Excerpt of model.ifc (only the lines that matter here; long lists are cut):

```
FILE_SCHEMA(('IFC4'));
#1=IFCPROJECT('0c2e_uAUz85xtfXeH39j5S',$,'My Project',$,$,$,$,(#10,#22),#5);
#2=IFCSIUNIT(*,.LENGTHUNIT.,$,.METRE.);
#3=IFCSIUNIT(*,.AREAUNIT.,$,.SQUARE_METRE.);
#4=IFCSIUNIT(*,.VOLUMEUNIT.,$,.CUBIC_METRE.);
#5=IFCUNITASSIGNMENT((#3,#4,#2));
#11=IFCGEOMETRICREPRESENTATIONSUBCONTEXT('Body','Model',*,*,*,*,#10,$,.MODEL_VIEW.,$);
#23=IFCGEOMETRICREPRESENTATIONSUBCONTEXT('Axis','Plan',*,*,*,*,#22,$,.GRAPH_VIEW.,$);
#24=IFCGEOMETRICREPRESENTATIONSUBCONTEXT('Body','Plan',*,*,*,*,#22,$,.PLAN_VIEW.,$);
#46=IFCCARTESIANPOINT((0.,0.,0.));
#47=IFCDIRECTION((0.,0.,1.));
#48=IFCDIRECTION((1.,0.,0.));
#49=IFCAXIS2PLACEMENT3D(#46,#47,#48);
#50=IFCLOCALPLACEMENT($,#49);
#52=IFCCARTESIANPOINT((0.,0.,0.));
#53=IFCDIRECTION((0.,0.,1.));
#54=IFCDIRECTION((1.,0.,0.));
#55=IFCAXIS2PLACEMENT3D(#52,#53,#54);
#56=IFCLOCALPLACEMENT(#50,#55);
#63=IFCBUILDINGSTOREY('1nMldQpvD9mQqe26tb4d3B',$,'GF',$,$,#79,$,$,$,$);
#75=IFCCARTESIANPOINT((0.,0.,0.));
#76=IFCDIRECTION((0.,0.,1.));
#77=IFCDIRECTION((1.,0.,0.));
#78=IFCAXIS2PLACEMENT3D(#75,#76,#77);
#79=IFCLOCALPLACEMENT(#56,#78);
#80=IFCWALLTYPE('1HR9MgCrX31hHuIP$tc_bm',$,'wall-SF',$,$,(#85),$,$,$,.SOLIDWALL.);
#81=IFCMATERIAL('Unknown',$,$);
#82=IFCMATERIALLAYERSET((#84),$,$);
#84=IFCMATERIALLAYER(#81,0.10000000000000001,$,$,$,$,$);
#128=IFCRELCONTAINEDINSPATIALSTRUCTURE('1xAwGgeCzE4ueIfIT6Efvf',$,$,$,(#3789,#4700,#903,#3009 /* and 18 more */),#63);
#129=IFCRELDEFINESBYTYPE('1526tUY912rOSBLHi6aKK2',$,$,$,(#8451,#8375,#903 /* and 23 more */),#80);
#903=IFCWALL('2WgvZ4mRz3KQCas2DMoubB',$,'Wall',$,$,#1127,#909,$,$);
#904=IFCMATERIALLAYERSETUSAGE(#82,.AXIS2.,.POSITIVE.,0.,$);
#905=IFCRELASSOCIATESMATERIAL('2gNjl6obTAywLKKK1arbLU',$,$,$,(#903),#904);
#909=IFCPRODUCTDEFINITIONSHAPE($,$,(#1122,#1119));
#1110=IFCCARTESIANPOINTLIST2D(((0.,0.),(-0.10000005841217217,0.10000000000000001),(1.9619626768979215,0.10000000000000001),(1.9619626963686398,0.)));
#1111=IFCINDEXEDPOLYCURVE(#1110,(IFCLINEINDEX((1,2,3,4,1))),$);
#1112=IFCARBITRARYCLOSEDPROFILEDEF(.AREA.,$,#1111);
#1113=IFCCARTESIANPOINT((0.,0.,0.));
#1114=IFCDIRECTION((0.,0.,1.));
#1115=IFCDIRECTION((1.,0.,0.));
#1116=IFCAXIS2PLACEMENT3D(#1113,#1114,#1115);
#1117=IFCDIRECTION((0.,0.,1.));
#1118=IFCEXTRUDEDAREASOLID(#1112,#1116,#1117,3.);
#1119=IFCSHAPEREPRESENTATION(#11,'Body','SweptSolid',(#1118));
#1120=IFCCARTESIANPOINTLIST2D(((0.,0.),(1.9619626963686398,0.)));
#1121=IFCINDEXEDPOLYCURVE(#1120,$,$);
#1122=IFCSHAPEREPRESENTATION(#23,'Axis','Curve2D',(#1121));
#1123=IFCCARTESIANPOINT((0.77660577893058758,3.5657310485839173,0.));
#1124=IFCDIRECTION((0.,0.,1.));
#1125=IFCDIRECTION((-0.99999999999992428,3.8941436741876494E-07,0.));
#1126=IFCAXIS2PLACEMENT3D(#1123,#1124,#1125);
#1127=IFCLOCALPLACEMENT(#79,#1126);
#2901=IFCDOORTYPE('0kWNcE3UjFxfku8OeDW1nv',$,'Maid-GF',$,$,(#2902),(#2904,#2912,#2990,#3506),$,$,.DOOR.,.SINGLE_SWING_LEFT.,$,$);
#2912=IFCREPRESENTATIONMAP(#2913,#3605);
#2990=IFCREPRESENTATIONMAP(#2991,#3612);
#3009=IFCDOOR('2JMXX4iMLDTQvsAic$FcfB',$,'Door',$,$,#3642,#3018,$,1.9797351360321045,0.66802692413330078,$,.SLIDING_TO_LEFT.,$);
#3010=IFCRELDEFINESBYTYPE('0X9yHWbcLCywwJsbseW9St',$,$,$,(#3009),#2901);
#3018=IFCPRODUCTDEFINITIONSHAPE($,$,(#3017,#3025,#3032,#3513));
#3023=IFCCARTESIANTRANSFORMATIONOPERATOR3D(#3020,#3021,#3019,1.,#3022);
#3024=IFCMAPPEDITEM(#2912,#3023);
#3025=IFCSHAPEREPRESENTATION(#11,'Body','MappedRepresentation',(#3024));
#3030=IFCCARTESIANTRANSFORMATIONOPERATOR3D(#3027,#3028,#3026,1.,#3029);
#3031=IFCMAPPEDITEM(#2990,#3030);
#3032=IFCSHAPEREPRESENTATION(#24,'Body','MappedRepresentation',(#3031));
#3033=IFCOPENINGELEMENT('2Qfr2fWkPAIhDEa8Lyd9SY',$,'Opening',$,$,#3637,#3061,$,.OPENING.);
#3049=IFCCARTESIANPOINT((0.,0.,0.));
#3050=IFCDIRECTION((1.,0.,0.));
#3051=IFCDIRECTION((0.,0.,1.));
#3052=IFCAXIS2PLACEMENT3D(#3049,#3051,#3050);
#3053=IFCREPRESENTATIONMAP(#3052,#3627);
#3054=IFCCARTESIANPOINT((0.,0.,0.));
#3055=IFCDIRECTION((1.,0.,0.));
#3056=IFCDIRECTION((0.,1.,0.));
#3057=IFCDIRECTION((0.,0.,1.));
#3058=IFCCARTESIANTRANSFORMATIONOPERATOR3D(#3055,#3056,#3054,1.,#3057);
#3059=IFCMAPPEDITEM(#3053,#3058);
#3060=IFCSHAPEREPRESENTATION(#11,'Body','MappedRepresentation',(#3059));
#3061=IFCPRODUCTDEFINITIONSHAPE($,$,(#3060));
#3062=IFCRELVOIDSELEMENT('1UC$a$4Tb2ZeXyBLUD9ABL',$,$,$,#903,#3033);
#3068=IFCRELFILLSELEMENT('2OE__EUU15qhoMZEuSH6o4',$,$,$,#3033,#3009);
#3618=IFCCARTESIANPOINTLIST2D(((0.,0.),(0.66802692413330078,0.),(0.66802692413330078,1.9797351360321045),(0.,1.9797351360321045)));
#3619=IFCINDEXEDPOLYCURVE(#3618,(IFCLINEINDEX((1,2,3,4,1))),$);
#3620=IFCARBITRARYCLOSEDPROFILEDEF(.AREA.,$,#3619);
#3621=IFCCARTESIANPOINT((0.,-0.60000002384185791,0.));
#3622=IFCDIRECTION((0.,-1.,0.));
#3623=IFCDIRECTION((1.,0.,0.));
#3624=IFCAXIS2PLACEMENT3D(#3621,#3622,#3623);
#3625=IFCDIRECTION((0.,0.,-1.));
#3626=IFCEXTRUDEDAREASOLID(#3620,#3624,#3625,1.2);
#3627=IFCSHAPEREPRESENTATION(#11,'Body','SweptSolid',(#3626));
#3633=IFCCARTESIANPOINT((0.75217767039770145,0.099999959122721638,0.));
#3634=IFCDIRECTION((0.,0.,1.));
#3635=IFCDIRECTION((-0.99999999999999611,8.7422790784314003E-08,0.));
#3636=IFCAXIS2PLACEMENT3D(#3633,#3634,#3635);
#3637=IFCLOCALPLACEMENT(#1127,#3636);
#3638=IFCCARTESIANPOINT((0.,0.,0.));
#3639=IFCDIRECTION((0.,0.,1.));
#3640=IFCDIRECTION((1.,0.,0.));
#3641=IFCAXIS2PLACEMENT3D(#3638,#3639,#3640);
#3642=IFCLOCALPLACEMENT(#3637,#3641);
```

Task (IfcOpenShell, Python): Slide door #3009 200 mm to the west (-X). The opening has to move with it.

```python
import ifcopenshell
import ifcopenshell.api.geometry
import ifcopenshell.util.placement
import ifcopenshell.util.unit

model = ifcopenshell.open("model.ifc")
unit_scale = ifcopenshell.util.unit.calculate_unit_scale(model)

door = model.by_guid("2JMXX4iMLDTQvsAic$FcfB")
opening = door.FillsVoids[0].RelatingOpeningElement
wall = opening.VoidsElements[0].RelatingBuildingElement

wall_matrix = ifcopenshell.util.placement.get_local_placement(wall.ObjectPlacement)
shift = wall_matrix[:3, 0] * 0.2 / unit_scale
before = ifcopenshell.util.placement.get_local_placement(door.ObjectPlacement)[:3, 3].copy()

# The door is placed relative to its opening, so it follows when the opening moves.
matrix = ifcopenshell.util.placement.get_local_placement(opening.ObjectPlacement)
matrix[:3, 3] += shift
ifcopenshell.api.geometry.edit_object_placement(
    model, product=opening, matrix=matrix, is_si=False, should_transform_children=True
)

after = ifcopenshell.util.placement.get_local_placement(door.ObjectPlacement)[:3, 3]
print("door moved by", (after - before).round(3) + 0.0)

model.write("model_rev.ifc")
```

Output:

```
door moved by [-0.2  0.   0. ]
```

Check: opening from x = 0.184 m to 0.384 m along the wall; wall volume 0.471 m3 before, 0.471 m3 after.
